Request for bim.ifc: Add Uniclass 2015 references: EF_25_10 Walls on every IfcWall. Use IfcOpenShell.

First a look at what the model holds.

```python
import ifcopenshell

model = ifcopenshell.open("bim.ifc")
print(model.schema)
print("classifications:", [c.Name for c in model.by_type("IfcClassification")])
for ifc_class in ("IfcDoor", "IfcRoof", "IfcStair", "IfcWall", "IfcWindow"):
    print(ifc_class, len(model.by_type(ifc_class)))
```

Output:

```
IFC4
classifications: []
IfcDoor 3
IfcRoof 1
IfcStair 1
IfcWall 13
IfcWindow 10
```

```python
import ifcopenshell
import ifcopenshell.api.classification

model = ifcopenshell.open("bim.ifc")

system = ifcopenshell.api.classification.add_classification(model, classification="Uniclass 2015")

codes = {
    "IfcWall": ("EF_25_10", "Walls"),
}
for ifc_class, (code, name) in codes.items():
    products = model.by_type(ifc_class)
    ifcopenshell.api.classification.add_reference(
        model, products=products, classification=system, identification=code, name=name
    )
    print(code, len(products))

model.write("bim_v2.ifc")
```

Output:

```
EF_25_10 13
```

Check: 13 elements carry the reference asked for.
